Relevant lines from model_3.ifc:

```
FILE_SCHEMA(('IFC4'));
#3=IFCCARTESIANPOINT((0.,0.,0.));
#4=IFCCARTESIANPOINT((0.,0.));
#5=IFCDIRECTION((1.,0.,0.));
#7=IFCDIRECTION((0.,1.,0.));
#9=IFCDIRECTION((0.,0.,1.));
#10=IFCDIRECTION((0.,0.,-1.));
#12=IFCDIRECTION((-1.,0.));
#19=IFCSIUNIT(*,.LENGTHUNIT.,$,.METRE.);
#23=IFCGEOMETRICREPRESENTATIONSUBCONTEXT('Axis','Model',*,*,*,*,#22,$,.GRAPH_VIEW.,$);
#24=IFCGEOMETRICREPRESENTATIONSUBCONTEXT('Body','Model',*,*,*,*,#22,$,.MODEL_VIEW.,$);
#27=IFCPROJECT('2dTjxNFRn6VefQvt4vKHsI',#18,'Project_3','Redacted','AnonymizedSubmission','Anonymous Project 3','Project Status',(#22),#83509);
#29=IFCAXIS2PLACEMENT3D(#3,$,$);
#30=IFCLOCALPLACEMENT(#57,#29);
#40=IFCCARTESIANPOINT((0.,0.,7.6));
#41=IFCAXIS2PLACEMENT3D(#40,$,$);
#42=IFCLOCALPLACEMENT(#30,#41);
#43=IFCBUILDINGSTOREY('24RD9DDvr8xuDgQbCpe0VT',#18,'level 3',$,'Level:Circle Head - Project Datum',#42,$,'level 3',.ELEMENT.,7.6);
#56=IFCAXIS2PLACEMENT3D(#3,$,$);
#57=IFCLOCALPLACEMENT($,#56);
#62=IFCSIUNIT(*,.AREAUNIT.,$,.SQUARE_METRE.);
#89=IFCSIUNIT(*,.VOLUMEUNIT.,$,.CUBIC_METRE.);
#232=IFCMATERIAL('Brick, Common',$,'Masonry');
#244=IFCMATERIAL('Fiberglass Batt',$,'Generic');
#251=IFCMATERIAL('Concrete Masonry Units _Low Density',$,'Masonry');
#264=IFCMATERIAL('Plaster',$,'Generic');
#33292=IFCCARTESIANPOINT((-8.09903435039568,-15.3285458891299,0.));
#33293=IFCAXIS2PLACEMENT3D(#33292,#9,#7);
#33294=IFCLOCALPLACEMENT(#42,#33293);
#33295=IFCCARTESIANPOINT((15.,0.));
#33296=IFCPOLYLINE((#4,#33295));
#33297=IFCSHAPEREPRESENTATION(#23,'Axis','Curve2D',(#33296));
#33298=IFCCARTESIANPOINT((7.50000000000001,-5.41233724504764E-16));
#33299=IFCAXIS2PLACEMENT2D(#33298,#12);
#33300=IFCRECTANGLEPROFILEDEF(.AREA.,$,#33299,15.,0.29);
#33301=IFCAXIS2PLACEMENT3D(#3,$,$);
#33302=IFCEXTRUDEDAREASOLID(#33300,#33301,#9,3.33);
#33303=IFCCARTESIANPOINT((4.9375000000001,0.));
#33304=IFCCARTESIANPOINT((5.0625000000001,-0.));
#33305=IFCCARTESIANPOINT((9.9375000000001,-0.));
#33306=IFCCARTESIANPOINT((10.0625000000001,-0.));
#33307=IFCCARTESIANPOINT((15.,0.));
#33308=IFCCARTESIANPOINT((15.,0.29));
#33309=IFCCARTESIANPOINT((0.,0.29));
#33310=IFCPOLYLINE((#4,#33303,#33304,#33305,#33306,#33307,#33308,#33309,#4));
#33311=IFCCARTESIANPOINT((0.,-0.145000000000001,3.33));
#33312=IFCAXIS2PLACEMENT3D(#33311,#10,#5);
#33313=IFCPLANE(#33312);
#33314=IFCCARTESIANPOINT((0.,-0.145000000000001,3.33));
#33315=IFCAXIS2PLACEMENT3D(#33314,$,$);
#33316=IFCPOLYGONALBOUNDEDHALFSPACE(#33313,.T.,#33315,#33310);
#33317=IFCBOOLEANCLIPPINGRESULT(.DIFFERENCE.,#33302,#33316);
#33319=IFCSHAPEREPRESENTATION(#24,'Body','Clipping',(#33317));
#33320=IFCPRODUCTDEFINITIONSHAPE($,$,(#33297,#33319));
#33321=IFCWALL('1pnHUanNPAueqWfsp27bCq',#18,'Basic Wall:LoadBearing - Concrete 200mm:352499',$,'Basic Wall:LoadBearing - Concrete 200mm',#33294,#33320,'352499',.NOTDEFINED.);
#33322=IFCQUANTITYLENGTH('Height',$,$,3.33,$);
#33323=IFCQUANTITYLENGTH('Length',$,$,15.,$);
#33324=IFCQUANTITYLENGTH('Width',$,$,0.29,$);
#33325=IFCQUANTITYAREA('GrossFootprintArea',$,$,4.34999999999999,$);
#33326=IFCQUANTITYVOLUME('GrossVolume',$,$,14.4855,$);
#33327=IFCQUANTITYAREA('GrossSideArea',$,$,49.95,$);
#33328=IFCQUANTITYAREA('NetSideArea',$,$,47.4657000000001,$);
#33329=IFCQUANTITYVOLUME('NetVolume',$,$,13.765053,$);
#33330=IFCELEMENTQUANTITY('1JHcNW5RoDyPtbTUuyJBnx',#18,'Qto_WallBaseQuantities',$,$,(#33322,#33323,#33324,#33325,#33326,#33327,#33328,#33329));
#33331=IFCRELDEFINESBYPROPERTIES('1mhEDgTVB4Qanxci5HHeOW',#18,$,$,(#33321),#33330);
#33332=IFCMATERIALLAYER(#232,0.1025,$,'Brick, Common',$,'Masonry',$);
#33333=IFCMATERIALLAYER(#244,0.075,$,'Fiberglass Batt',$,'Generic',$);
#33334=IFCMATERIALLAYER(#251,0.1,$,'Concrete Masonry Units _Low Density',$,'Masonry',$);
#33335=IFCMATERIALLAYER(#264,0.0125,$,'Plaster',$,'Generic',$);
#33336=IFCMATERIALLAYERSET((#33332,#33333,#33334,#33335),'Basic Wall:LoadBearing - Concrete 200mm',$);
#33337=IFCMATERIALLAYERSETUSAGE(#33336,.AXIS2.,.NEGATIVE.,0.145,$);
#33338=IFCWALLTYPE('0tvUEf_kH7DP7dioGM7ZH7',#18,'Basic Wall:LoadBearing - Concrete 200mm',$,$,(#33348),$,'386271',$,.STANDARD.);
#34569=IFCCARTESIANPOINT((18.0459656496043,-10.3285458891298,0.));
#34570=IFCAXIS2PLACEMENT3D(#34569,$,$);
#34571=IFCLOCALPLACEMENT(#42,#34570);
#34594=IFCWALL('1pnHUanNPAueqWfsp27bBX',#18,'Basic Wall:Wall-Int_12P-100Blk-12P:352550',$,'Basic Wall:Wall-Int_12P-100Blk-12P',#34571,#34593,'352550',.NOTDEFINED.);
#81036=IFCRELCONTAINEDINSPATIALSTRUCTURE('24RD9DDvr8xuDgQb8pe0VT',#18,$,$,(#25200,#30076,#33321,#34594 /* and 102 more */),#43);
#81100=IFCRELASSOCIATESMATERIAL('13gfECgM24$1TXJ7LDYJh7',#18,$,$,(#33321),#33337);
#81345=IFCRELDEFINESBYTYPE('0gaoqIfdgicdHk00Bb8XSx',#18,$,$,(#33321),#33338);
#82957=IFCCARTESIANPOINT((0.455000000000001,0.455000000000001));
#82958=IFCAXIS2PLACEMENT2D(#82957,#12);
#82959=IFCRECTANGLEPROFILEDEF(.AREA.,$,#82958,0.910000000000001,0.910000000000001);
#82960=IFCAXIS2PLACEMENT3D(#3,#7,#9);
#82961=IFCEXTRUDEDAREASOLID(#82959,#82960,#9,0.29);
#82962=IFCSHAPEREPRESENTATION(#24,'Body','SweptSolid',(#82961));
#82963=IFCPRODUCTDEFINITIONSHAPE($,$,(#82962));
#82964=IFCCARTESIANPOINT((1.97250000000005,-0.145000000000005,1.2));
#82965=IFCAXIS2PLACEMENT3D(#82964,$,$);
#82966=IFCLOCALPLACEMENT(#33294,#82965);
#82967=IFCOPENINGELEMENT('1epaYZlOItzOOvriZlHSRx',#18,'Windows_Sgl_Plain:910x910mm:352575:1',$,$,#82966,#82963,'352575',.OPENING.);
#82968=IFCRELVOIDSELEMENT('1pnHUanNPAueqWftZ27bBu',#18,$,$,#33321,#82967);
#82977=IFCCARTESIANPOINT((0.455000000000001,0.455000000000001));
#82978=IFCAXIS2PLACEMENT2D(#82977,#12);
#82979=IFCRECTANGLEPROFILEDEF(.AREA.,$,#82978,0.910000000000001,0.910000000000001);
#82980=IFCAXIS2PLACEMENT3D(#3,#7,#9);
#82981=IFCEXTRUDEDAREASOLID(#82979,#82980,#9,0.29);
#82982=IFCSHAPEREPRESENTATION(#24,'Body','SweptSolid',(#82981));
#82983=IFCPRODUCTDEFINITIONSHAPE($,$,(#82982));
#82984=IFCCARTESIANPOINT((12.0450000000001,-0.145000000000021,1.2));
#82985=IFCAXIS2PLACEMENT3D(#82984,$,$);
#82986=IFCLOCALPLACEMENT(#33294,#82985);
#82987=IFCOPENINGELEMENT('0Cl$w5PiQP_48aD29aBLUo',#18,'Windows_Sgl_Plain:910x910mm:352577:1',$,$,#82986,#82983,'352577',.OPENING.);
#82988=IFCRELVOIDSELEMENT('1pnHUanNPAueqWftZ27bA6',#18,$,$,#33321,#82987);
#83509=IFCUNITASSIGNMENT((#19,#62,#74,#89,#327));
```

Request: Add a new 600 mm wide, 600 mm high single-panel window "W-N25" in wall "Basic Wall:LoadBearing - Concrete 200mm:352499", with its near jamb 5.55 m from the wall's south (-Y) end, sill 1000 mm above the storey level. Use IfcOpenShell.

```python
import numpy as np
import ifcopenshell
import ifcopenshell.api.feature
import ifcopenshell.api.geometry
import ifcopenshell.api.pset
import ifcopenshell.api.root
import ifcopenshell.api.spatial
import ifcopenshell.geom
import ifcopenshell.util.element
import ifcopenshell.util.placement
import ifcopenshell.util.representation
import ifcopenshell.util.shape
import ifcopenshell.util.unit

model = ifcopenshell.open("model_3.ifc")
unit_scale = ifcopenshell.util.unit.calculate_unit_scale(model)
area_scale = ifcopenshell.util.unit.calculate_unit_scale(model, "AREAUNIT")
volume_scale = ifcopenshell.util.unit.calculate_unit_scale(model, "VOLUMEUNIT")
settings = ifcopenshell.geom.settings()


def volume(element):
    """Net volume in cubic metres, openings subtracted."""
    shape = ifcopenshell.geom.create_shape(settings, element)
    return ifcopenshell.util.shape.get_volume(shape.geometry)


wall = model.by_guid("1pnHUanNPAueqWfsp27bCq")
storey = ifcopenshell.util.element.get_container(wall, ifc_class="IfcBuildingStorey")
context = ifcopenshell.util.representation.get_context(model, "Model", "Body", "MODEL_VIEW")
before = volume(wall)

width, height, from_end, sill = 0.6, 0.6, 5.55, 1  # metres

# The wall runs along its own X axis, and the end named is its -X end.
wall_shape = ifcopenshell.geom.create_shape(settings, wall)
x, y, z = ifcopenshell.util.shape.get_vertices(wall_shape.geometry).T
start = x.min() + from_end
face, thickness = float(y.min()), float(y.max() - y.min())
wall_matrix = ifcopenshell.util.placement.get_local_placement(wall.ObjectPlacement)
level = ifcopenshell.util.placement.get_local_placement(storey.ObjectPlacement)[2, 3]


def in_wall(x, y):
    """Placement at x, y metres in the wall's axes, at sill height."""
    matrix = wall_matrix.copy()
    matrix[:, 3] = wall_matrix @ np.array([x / unit_scale, y / unit_scale, 0.0, 1.0])
    matrix[2, 3] = level + sill / unit_scale
    return matrix


# Opening: a box that overshoots both wall faces by 50 mm.
opening = ifcopenshell.api.root.create_entity(model, ifc_class="IfcOpeningElement", predefined_type="OPENING")
box = ifcopenshell.api.geometry.add_wall_representation(
    model, context=context, length=width, height=height, thickness=thickness + 0.1
)
ifcopenshell.api.geometry.assign_representation(model, product=opening, representation=box)
ifcopenshell.api.geometry.edit_object_placement(model, product=opening, matrix=in_wall(start, face - 0.05), is_si=False)
ifcopenshell.api.feature.add_feature(model, feature=opening, element=wall)

window = ifcopenshell.api.root.create_entity(model, ifc_class="IfcWindow", name="W-N25", predefined_type="WINDOW")
window.OverallWidth, window.OverallHeight = width / unit_scale, height / unit_scale
window.PartitioningType = "SINGLE_PANEL"
body = ifcopenshell.api.geometry.add_window_representation(
    model,
    context=context,
    overall_width=window.OverallWidth,
    overall_height=window.OverallHeight,
    partition_type="SINGLE_PANEL",
)
ifcopenshell.api.geometry.assign_representation(model, product=window, representation=body)
ifcopenshell.api.spatial.assign_container(model, products=[window], relating_structure=storey)
ifcopenshell.api.feature.add_filling(model, opening=opening, element=window)

# Centre the window in the wall's thickness.
ifcopenshell.api.geometry.edit_object_placement(model, product=window, matrix=in_wall(start, face), is_si=False)
window_shape = ifcopenshell.geom.create_shape(settings, window)
depth = ifcopenshell.util.shape.get_vertices(window_shape.geometry)[:, 1]
offset = face + thickness / 2 - (depth.min() + depth.max()) / 2
ifcopenshell.api.geometry.edit_object_placement(model, product=window, matrix=in_wall(start, offset), is_si=False)

after = volume(wall)

# Update the wall's stored quantities.
qto = model.by_id(ifcopenshell.util.element.get_pset(wall, "Qto_WallBaseQuantities", should_inherit=False)["id"])
ifcopenshell.api.pset.edit_qto(model, qto=qto, properties={
    "NetSideArea": after / thickness / area_scale,
    "NetVolume": after / volume_scale,
})

print(f"wall volume {before:.3f} -> {after:.3f} m3")

model.write("model_3-out.ifc")
```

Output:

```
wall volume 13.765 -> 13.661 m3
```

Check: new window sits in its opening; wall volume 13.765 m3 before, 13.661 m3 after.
